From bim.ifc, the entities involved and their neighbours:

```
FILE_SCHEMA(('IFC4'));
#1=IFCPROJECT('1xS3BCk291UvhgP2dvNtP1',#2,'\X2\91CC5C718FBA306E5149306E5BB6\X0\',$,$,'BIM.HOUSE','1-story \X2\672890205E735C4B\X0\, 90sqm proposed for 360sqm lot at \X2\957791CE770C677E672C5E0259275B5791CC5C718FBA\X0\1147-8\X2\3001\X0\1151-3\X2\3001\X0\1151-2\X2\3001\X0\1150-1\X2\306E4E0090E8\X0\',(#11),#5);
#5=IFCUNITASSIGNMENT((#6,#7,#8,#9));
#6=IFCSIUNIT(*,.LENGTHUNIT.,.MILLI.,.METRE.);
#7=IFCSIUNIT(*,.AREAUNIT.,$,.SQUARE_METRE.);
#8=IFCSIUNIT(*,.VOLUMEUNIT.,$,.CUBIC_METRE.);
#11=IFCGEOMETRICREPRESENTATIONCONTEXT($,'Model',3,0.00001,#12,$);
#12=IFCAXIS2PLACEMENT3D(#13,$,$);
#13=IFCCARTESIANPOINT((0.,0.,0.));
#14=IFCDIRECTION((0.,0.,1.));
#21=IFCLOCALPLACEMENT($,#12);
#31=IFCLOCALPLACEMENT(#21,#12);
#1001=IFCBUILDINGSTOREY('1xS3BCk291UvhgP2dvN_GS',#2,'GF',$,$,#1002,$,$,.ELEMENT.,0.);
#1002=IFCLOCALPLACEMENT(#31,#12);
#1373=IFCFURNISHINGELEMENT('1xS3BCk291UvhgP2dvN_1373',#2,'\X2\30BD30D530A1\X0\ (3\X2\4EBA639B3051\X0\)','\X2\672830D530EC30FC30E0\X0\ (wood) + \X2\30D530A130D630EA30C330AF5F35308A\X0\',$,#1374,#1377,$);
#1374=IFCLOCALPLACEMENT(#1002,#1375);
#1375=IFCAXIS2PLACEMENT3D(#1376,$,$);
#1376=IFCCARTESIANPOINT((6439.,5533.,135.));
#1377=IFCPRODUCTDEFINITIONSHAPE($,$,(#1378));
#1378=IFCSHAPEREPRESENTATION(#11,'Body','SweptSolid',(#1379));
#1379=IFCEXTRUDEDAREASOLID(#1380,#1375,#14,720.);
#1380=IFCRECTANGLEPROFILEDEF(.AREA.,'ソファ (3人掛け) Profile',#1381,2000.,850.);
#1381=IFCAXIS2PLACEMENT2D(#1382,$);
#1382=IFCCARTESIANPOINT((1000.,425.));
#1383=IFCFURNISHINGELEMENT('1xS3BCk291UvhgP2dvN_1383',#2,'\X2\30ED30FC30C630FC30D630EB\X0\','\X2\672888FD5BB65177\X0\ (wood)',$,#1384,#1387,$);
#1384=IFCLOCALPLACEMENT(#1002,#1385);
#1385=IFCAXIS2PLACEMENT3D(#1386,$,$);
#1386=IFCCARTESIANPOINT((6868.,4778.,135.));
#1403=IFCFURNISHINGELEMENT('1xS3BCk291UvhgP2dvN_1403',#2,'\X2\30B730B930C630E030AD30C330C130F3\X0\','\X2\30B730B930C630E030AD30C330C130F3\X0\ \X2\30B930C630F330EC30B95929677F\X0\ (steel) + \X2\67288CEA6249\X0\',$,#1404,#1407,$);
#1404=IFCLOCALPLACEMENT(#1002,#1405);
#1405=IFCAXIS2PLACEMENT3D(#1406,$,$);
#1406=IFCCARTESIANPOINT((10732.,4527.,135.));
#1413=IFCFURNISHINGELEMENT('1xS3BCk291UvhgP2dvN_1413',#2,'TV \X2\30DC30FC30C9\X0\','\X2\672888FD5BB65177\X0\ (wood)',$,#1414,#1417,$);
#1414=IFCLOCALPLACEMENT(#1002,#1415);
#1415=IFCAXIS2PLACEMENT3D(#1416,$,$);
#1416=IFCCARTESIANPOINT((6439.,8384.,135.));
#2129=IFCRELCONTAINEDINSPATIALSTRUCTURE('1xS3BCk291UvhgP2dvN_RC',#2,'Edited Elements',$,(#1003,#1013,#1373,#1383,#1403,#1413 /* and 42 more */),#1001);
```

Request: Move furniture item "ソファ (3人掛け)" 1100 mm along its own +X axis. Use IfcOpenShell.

```python
import ifcopenshell
import ifcopenshell.api.geometry
import ifcopenshell.util.placement
import ifcopenshell.util.unit

model = ifcopenshell.open("bim.ifc")
unit_scale = ifcopenshell.util.unit.calculate_unit_scale(model)

item = model.by_id(1373)
matrix = ifcopenshell.util.placement.get_local_placement(item.ObjectPlacement)
matrix[:3, 3] += matrix[:3, 0] * 1.1 / unit_scale
ifcopenshell.api.geometry.edit_object_placement(model, product=item, matrix=matrix, is_si=False)

print(ifcopenshell.util.placement.get_local_placement(item.ObjectPlacement).round(3) + 0.0)

model.write("bim_edited.ifc")
```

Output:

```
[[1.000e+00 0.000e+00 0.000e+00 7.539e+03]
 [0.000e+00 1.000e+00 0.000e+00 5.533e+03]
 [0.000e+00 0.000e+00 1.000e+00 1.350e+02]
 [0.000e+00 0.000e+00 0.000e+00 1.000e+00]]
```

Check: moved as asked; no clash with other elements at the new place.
